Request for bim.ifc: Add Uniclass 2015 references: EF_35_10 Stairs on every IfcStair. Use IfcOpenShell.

First a look at what the model holds.

```python
import ifcopenshell

model = ifcopenshell.open("bim.ifc")
print(model.schema)
print("classifications:", [c.Name for c in model.by_type("IfcClassification")])
for ifc_class in ("IfcDoor", "IfcRoof", "IfcStair", "IfcWall", "IfcWindow"):
    print(ifc_class, len(model.by_type(ifc_class)))
```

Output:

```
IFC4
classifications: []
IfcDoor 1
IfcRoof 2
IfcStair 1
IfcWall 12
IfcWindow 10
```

```python
import ifcopenshell
import ifcopenshell.api.classification

model = ifcopenshell.open("bim.ifc")

system = ifcopenshell.api.classification.add_classification(model, classification="Uniclass 2015")

codes = {
    "IfcStair": ("EF_35_10", "Stairs"),
}
for ifc_class, (code, name) in codes.items():
    products = model.by_type(ifc_class)
    ifcopenshell.api.classification.add_reference(
        model, products=products, classification=system, identification=code, name=name
    )
    print(code, len(products))

model.write("bim_rev.ifc")
```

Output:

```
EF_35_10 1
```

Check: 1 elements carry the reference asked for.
